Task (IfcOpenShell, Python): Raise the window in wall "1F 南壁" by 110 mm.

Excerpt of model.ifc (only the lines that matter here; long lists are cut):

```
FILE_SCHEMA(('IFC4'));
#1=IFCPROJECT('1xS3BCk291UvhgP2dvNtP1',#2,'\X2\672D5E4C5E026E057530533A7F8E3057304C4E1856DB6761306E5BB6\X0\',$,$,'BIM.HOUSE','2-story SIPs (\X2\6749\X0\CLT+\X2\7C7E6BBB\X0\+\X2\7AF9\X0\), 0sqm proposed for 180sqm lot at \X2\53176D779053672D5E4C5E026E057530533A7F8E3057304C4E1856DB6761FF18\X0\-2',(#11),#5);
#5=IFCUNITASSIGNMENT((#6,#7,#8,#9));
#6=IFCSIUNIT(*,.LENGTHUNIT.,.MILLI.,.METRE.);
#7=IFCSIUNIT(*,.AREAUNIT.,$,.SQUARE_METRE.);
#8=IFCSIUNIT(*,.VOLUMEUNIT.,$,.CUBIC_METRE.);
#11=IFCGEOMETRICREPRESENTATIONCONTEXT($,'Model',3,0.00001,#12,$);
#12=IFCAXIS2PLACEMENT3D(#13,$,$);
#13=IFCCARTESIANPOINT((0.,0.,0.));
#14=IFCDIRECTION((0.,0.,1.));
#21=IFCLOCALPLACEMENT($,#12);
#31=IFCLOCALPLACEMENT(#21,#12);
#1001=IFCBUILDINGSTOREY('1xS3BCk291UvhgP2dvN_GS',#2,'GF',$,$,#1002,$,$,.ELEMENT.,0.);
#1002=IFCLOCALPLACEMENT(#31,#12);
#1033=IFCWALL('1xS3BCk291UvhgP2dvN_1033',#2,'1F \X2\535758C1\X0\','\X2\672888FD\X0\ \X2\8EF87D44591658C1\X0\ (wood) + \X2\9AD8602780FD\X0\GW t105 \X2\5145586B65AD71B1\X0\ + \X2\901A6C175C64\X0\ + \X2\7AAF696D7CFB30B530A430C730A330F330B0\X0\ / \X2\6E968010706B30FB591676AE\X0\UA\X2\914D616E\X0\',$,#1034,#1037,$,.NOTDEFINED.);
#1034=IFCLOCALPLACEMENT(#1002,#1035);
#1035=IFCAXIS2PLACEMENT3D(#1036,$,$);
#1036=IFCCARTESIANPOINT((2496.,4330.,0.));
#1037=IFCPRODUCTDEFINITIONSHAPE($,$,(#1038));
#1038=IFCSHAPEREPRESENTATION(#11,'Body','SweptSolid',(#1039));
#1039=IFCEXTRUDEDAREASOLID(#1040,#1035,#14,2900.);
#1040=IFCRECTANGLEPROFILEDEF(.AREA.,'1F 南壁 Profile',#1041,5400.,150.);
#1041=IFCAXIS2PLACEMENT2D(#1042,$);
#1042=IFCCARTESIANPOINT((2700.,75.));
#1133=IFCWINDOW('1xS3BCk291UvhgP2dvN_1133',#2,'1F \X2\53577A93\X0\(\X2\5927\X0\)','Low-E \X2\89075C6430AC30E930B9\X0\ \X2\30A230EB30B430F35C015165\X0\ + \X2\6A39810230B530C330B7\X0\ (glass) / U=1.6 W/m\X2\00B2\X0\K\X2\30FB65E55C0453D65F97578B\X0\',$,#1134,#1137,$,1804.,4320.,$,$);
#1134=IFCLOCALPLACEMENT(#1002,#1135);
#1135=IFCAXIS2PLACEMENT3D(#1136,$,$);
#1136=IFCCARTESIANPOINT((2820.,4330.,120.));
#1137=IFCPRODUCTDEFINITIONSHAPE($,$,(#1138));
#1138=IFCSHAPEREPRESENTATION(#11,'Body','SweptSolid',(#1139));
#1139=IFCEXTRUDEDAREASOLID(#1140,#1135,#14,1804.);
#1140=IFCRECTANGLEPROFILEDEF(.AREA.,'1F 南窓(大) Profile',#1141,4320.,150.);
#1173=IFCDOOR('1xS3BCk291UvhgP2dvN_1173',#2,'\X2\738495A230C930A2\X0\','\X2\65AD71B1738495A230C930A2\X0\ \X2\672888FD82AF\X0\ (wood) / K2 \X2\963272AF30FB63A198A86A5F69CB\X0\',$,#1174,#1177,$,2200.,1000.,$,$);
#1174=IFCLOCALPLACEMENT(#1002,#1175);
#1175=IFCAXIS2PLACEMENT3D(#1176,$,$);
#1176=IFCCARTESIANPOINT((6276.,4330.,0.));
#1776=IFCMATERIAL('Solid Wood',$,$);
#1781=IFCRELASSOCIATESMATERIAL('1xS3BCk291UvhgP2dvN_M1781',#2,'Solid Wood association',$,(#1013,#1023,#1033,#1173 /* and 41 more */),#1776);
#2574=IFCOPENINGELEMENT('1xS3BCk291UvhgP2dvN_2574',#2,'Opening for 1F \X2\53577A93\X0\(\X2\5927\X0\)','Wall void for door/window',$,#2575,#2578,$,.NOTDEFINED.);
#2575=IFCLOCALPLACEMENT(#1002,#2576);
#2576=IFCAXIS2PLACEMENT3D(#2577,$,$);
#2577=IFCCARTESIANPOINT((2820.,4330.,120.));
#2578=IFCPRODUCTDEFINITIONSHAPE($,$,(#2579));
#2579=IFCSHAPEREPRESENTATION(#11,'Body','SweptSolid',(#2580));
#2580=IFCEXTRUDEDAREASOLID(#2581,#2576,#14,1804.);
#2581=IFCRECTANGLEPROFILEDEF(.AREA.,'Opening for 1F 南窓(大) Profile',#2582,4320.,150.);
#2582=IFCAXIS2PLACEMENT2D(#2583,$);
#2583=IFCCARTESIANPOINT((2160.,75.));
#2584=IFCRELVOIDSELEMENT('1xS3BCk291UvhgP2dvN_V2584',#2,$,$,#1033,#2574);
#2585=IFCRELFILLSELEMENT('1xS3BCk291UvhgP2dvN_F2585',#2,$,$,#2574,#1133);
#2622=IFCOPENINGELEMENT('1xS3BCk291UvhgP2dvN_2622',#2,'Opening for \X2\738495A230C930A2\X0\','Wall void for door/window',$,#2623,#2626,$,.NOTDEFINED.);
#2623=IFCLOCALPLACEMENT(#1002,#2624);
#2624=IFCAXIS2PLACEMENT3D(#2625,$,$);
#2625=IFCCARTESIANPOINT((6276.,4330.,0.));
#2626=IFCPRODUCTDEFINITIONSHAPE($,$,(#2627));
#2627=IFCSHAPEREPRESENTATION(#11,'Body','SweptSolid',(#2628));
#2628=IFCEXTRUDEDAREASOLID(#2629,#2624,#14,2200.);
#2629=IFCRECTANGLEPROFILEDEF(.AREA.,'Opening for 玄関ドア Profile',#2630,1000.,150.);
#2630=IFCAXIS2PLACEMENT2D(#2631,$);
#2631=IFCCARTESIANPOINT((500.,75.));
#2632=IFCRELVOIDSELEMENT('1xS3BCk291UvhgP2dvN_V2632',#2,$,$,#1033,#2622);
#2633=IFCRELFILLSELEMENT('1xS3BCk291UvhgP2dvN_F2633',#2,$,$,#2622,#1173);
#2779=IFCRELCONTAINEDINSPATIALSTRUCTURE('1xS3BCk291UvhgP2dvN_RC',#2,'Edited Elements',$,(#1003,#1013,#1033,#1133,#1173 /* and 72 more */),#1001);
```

```python
import numpy as np
import ifcopenshell
import ifcopenshell.api.geometry
import ifcopenshell.util.placement
import ifcopenshell.util.unit

model = ifcopenshell.open("model.ifc")
unit_scale = ifcopenshell.util.unit.calculate_unit_scale(model)

window = model.by_guid("1xS3BCk291UvhgP2dvN_1133")
opening = window.FillsVoids[0].RelatingOpeningElement
dz = 0.11 / unit_scale

shift = np.array([0.0, 0.0, dz])
# The window is not placed relative to its opening, so move both.
for product in (opening, window):
    matrix = ifcopenshell.util.placement.get_local_placement(product.ObjectPlacement)
    matrix[:3, 3] += shift
    ifcopenshell.api.geometry.edit_object_placement(model, product=product, matrix=matrix, is_si=False)

print(f"moved by {dz * unit_scale:+.3f} m")

model.write("model_v2.ifc")
```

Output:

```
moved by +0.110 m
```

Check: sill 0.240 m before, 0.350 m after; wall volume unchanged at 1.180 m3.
